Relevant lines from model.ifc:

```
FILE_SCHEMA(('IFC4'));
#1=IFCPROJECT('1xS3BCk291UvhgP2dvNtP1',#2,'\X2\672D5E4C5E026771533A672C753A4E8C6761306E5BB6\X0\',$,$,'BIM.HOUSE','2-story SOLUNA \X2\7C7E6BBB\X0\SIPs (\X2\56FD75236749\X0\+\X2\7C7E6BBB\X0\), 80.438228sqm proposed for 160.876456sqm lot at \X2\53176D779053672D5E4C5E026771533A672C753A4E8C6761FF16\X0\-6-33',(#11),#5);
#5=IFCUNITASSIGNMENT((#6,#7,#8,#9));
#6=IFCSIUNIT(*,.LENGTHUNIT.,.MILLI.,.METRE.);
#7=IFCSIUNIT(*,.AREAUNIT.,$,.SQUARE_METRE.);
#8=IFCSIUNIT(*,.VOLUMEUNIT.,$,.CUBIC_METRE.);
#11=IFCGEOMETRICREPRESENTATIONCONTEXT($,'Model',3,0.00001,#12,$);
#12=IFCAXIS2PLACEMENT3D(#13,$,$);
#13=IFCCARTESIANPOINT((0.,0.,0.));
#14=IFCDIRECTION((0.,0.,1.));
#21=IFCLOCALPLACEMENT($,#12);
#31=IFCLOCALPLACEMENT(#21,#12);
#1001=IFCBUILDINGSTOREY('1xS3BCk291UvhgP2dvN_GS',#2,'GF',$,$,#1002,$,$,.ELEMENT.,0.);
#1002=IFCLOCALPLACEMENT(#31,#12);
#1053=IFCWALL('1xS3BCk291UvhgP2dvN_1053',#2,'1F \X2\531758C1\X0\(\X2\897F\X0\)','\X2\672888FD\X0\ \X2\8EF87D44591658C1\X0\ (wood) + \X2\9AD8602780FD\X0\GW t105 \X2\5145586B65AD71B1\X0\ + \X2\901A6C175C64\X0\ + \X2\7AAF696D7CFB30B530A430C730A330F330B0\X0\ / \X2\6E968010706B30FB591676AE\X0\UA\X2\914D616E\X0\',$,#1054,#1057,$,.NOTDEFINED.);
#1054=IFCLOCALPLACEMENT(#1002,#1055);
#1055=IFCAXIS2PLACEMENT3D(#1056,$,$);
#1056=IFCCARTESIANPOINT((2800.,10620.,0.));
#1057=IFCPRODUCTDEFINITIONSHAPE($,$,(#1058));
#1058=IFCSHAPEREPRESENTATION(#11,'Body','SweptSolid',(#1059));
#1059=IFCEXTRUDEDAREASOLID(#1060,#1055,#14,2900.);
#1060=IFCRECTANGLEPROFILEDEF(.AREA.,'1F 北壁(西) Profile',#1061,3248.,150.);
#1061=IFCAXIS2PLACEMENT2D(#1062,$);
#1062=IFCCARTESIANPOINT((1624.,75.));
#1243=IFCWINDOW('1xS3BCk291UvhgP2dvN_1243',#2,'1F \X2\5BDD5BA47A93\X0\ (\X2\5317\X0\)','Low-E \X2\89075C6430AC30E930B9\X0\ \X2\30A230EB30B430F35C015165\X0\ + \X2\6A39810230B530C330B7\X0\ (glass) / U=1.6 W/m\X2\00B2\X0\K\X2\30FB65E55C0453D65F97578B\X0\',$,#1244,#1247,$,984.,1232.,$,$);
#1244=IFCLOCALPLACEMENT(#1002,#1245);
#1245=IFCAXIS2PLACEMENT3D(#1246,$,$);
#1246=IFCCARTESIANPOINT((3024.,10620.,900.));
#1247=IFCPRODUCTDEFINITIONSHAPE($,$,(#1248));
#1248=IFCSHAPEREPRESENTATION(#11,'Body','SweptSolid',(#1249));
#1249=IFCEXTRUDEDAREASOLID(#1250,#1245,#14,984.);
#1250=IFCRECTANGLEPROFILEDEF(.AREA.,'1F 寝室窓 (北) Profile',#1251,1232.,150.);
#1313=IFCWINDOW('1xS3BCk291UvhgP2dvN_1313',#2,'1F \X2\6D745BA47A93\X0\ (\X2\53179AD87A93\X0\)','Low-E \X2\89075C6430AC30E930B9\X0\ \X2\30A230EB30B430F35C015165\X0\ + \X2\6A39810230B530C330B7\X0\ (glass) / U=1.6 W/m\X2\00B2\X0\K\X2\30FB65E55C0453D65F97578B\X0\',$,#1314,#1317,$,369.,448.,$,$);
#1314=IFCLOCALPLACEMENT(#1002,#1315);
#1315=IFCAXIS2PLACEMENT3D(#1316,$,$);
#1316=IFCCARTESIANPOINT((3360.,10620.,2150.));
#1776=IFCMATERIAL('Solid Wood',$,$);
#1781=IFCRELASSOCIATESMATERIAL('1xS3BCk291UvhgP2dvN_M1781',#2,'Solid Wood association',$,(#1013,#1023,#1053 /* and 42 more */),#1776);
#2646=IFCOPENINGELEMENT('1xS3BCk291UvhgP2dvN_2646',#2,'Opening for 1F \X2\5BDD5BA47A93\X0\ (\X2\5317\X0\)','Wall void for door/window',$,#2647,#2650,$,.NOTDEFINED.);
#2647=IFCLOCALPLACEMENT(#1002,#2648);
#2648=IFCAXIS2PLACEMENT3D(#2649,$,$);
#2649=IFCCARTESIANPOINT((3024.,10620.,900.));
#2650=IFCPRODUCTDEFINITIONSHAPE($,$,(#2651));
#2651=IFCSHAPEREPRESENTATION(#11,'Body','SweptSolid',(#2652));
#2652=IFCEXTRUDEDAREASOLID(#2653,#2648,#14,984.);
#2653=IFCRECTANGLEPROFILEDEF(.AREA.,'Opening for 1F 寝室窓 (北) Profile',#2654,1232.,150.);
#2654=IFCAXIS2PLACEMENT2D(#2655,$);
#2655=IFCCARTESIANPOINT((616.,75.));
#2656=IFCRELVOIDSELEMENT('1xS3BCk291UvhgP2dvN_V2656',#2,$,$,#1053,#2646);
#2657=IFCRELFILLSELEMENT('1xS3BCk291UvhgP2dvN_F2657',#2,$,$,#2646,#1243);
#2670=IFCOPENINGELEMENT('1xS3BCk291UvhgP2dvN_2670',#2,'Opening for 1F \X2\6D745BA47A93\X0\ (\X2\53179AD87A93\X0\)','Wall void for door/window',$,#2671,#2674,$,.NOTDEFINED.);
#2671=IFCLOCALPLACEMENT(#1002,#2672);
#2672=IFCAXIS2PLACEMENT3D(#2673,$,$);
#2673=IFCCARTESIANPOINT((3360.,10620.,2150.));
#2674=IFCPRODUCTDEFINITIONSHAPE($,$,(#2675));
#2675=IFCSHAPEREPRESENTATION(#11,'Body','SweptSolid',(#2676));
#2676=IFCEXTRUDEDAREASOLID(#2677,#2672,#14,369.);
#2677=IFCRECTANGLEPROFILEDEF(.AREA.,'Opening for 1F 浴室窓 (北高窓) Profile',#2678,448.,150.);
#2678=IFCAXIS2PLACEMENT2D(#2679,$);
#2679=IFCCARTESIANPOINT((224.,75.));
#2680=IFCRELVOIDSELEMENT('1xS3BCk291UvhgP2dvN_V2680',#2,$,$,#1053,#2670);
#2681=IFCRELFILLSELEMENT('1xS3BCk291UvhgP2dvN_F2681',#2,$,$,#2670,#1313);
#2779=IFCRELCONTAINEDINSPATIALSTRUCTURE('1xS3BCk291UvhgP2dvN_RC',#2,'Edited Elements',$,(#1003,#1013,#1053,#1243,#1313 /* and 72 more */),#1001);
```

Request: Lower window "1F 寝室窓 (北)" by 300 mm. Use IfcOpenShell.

```python
import numpy as np
import ifcopenshell
import ifcopenshell.api.geometry
import ifcopenshell.util.placement
import ifcopenshell.util.unit

model = ifcopenshell.open("model.ifc")
unit_scale = ifcopenshell.util.unit.calculate_unit_scale(model)

window = model.by_id(1243)
opening = window.FillsVoids[0].RelatingOpeningElement
dz = -300.0

shift = np.array([0.0, 0.0, dz])
# The window is not placed relative to its opening, so move both.
for product in (opening, window):
    matrix = ifcopenshell.util.placement.get_local_placement(product.ObjectPlacement)
    matrix[:3, 3] += shift
    ifcopenshell.api.geometry.edit_object_placement(model, product=product, matrix=matrix, is_si=False)

print(f"moved by {dz * unit_scale:+.3f} m")

model.write("model_v2.ifc")
```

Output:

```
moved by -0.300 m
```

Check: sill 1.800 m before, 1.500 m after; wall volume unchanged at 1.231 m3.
